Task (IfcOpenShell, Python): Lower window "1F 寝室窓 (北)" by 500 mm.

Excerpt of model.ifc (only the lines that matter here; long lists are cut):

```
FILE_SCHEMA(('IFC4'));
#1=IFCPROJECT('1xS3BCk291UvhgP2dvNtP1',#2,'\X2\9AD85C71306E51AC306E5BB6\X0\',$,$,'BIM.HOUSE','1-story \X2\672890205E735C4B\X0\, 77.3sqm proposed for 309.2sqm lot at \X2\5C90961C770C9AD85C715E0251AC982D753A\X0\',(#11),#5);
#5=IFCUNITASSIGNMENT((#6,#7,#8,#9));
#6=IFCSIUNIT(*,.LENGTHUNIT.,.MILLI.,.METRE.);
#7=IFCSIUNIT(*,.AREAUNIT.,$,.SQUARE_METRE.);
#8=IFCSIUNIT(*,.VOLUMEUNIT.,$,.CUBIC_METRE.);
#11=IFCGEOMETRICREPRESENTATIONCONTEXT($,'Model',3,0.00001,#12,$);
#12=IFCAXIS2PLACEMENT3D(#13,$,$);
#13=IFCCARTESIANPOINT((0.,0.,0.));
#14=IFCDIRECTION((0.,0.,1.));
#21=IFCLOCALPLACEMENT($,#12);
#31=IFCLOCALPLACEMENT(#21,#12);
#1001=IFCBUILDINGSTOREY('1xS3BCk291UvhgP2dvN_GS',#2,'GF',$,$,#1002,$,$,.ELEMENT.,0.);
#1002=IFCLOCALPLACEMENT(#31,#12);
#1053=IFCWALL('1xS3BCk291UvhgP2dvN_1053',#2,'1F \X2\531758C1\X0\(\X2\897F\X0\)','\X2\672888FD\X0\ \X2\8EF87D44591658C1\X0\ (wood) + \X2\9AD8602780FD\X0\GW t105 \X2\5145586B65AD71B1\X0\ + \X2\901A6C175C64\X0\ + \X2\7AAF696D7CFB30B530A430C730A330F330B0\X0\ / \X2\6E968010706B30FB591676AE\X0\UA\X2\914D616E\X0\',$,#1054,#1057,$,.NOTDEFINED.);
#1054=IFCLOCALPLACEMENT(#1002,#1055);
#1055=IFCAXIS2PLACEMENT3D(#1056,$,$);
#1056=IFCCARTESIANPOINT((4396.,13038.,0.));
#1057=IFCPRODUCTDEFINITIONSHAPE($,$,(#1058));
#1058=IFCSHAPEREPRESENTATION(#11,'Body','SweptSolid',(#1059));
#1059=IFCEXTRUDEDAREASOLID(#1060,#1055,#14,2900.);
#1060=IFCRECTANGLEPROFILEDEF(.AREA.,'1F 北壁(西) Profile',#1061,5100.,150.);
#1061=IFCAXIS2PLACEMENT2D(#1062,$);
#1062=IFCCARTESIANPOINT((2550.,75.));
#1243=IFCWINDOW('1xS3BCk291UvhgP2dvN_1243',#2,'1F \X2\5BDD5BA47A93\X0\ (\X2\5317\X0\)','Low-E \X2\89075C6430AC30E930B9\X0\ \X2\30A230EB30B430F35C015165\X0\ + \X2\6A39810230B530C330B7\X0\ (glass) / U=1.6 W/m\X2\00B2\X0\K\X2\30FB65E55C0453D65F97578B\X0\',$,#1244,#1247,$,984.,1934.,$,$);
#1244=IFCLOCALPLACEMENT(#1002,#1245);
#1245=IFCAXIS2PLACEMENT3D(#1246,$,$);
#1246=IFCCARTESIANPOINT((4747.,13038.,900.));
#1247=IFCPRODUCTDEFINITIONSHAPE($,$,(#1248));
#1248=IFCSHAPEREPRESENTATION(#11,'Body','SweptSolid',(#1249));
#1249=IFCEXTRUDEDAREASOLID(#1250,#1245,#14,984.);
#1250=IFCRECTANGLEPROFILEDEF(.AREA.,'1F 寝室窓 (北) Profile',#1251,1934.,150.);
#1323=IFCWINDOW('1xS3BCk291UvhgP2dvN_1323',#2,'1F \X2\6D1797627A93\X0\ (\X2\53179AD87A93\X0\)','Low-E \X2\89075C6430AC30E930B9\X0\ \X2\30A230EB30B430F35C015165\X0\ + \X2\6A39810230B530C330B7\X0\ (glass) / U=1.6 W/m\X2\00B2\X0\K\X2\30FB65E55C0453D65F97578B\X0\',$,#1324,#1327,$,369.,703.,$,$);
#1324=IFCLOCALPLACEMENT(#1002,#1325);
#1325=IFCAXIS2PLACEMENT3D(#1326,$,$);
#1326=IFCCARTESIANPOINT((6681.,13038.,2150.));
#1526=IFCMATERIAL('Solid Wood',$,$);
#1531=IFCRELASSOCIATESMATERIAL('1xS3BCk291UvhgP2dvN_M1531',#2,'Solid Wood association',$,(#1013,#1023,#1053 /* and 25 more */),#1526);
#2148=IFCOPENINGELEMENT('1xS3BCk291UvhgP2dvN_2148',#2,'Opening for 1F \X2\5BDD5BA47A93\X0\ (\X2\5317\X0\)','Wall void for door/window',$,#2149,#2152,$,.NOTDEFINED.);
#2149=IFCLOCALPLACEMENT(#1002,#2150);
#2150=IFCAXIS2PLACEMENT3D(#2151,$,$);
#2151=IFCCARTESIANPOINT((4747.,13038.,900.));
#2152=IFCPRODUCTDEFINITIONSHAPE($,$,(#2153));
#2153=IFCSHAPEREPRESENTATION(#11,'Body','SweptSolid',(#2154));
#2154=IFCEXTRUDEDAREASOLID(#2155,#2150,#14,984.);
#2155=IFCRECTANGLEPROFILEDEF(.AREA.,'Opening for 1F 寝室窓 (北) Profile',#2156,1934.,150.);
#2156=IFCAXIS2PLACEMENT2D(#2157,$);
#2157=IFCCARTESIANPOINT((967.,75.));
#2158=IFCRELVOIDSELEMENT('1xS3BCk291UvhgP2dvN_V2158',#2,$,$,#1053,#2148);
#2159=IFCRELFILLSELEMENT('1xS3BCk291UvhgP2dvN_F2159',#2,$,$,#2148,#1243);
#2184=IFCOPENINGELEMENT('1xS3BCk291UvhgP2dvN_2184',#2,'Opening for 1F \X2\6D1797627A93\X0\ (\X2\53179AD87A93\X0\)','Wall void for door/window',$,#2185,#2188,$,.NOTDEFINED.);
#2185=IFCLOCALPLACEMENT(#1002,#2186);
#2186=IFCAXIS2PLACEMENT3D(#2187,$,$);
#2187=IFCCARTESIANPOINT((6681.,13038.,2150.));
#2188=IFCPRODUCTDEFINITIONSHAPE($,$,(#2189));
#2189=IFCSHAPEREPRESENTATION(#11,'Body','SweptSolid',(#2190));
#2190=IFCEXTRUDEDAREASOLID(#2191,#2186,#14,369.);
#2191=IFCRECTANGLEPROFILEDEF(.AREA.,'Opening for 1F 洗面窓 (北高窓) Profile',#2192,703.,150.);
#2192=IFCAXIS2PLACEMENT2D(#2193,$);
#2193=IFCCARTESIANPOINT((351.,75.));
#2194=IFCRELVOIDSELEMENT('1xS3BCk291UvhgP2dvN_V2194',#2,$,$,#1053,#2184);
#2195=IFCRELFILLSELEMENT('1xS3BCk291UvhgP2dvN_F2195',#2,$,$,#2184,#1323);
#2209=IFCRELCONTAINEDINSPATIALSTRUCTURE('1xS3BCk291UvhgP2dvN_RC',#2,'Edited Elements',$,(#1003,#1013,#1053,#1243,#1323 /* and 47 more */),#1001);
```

```python
import numpy as np
import ifcopenshell
import ifcopenshell.api.geometry
import ifcopenshell.util.placement
import ifcopenshell.util.unit

model = ifcopenshell.open("model.ifc")
unit_scale = ifcopenshell.util.unit.calculate_unit_scale(model)

window = model.by_guid("1xS3BCk291UvhgP2dvN_1243")
opening = window.FillsVoids[0].RelatingOpeningElement
dz = -500.0

shift = np.array([0.0, 0.0, dz])
# The window is not placed relative to its opening, so move both.
for product in (opening, window):
    matrix = ifcopenshell.util.placement.get_local_placement(product.ObjectPlacement)
    matrix[:3, 3] += shift
    ifcopenshell.api.geometry.edit_object_placement(model, product=product, matrix=matrix, is_si=False)

print(f"moved by {dz * unit_scale:+.3f} m")

model.write("model_updated.ifc")
```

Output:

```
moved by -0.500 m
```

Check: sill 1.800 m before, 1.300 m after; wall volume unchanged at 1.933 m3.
